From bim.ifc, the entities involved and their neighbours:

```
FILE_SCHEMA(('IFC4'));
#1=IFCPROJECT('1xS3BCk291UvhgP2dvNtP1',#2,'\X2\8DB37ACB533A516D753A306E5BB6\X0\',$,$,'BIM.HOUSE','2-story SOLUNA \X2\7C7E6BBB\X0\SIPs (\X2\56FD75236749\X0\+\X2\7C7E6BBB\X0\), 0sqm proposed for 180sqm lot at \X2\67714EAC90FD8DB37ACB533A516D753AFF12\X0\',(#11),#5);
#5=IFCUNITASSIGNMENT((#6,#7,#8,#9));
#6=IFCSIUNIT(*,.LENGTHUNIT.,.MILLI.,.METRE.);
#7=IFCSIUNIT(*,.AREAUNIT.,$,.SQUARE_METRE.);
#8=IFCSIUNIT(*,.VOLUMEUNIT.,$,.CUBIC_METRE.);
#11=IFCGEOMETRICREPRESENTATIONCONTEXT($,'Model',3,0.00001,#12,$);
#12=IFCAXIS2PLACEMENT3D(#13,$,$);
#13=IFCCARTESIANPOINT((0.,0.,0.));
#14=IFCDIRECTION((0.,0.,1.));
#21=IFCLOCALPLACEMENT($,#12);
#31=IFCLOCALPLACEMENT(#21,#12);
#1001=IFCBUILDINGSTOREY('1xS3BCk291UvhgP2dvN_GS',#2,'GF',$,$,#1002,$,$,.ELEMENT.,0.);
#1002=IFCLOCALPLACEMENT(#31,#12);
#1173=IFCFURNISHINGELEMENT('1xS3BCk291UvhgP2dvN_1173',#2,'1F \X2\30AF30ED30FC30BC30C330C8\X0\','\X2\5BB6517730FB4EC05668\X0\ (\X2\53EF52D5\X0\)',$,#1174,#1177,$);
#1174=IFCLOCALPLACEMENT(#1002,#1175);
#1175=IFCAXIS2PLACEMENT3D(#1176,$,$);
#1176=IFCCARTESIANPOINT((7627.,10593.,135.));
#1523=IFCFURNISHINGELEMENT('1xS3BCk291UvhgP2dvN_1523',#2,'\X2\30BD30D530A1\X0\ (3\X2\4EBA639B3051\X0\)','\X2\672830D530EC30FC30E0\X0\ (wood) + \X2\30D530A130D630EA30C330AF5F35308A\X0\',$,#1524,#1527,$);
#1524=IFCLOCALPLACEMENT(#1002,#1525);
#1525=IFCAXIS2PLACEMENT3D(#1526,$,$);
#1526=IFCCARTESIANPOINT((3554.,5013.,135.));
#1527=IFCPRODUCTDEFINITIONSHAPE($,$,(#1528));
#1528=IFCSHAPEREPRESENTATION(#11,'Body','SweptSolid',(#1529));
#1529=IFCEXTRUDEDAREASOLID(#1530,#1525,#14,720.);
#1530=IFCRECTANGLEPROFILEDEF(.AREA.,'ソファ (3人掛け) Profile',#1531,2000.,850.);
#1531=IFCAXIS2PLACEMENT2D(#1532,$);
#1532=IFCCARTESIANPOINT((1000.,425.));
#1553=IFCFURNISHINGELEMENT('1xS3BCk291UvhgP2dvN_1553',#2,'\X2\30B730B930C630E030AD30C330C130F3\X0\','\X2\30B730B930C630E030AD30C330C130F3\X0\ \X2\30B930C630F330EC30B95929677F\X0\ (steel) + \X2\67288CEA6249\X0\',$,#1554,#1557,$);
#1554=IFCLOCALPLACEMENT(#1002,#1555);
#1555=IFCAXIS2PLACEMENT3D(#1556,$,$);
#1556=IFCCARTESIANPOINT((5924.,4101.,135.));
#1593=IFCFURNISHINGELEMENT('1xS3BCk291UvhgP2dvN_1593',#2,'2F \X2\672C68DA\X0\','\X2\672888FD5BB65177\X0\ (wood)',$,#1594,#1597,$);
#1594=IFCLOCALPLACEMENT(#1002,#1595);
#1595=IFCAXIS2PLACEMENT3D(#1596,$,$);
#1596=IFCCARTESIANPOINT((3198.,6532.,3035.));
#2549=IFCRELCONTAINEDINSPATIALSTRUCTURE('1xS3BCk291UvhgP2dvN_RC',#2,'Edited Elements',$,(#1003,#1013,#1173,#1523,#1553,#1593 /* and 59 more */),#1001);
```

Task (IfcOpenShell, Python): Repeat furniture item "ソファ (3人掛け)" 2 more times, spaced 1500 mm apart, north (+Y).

```python
import numpy as np
import ifcopenshell
import ifcopenshell.api.geometry
import ifcopenshell.api.root
import ifcopenshell.util.element
import ifcopenshell.util.placement
import ifcopenshell.util.unit

model = ifcopenshell.open("bim.ifc")
unit_scale = ifcopenshell.util.unit.calculate_unit_scale(model)


def reuse_history(source, copy):
    """copy_class also copies each property set's owner history, people and application; keep the originals."""
    for rel in copy.IsDefinedBy:
        if rel.is_a("IfcRelDefinesByProperties") and (history := rel.RelatingPropertyDefinition.OwnerHistory):
            rel.RelatingPropertyDefinition.OwnerHistory = source.OwnerHistory
            ifcopenshell.util.element.remove_deep2(model, history)


source = model.by_id(1523)
base = ifcopenshell.util.placement.get_local_placement(source.ObjectPlacement)
step = np.array([0.0, 1.0, 0.0]) * 1.5 / unit_scale

for i in range(1, 3):
    copy = ifcopenshell.api.root.copy_class(model, product=source)
    copy.Representation = ifcopenshell.util.element.copy_deep(
        model, source.Representation, exclude=["IfcGeometricRepresentationContext", "IfcRepresentationMap"]
    )
    reuse_history(source, copy)
    matrix = base.copy()
    matrix[:3, 3] += i * step
    print("added at", matrix[:3, 3].round(3) + 0.0)
    ifcopenshell.api.geometry.edit_object_placement(model, product=copy, matrix=matrix, is_si=False)

model.write("bim_v2.ifc")
```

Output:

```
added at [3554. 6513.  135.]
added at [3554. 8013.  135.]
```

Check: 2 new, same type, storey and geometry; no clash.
